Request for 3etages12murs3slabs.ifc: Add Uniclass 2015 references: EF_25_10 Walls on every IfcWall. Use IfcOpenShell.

First a look at what the model holds.

```python
import ifcopenshell

model = ifcopenshell.open("3etages12murs3slabs.ifc")
print(model.schema)
print("classifications:", [c.Name for c in model.by_type("IfcClassification")])
for ifc_class in ("IfcDoor", "IfcRoof", "IfcStair", "IfcWall", "IfcWindow"):
    print(ifc_class, len(model.by_type(ifc_class)))
```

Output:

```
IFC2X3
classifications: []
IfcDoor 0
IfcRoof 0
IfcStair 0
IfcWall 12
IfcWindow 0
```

```python
import ifcopenshell
import ifcopenshell.api.classification

model = ifcopenshell.open("3etages12murs3slabs.ifc")

# IFC2X3 requires Source and Edition and has no link from the project to the system.
system = model.create_entity("IfcClassification", Source="NBS", Edition="2015", Name="Uniclass 2015")

codes = {
    "IfcWall": ("EF_25_10", "Walls"),
}
for ifc_class, (code, name) in codes.items():
    products = model.by_type(ifc_class)
    ifcopenshell.api.classification.add_reference(
        model, products=products, classification=system, identification=code, name=name
    )
    print(code, len(products))

model.write("3etages12murs3slabs-out.ifc")
```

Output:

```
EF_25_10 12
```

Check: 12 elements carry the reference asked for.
